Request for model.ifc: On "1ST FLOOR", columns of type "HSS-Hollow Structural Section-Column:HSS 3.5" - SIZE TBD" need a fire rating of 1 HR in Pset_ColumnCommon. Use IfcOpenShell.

First a look at what the model holds.

```python
import ifcopenshell
import ifcopenshell.util.element

model = ifcopenshell.open("model.ifc")
print(model.schema)
storey = next(s for s in model.by_type("IfcBuildingStorey") if s.Name == "1ST FLOOR")
columns = [e for e in ifcopenshell.util.element.get_decomposition(storey) if e.is_a("IfcColumn")]
seen = {}
for e in columns:
    element_type = ifcopenshell.util.element.get_type(e)
    key = (element_type.Name if element_type != e and element_type else None, ifcopenshell.util.element.get_pset(e, "Pset_ColumnCommon", "FireRating"))
    seen[key] = seen.get(key, 0) + 1
for (name, value), count in sorted(seen.items(), key=str):
    print(count, "x", name, "|", value)
```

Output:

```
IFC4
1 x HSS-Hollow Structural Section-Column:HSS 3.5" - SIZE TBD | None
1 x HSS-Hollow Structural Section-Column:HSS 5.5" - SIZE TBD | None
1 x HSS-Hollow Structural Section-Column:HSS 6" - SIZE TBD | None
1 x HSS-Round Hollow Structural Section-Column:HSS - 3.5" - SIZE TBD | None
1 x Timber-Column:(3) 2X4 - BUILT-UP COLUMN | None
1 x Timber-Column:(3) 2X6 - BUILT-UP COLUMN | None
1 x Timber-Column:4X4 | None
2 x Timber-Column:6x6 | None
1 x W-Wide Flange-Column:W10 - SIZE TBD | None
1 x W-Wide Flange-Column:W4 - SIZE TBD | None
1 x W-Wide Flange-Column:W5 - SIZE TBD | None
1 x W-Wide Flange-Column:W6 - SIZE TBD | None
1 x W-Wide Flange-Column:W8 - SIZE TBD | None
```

```python
import ifcopenshell
import ifcopenshell.api.pset
import ifcopenshell.util.element

model = ifcopenshell.open("model.ifc")

storey = next(s for s in model.by_type("IfcBuildingStorey") if s.Name == "1ST FLOOR")
columns = [e for e in ifcopenshell.util.element.get_decomposition(storey) if e.is_a("IfcColumn")]

count = 0
for e in columns:
    element_type = ifcopenshell.util.element.get_type(e)
    if element_type in (None, e) or element_type.Name != 'HSS-Hollow Structural Section-Column:HSS 3.5" - SIZE TBD':
        continue
    # add_pset returns the element's existing set when there is one.
    pset = ifcopenshell.api.pset.add_pset(model, product=e, name="Pset_ColumnCommon")
    ifcopenshell.api.pset.edit_pset(model, pset=pset, properties={"FireRating": "1 HR"})
    count += 1

print(count, "columns updated")

model.write("model_updated.ifc")
```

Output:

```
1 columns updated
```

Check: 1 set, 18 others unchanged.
